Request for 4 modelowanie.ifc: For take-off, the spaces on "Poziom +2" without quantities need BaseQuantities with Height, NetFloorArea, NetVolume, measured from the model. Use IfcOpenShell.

First a look at what the model holds.

```python
import ifcopenshell
import ifcopenshell.util.element
import ifcopenshell.util.unit

model = ifcopenshell.open("4 modelowanie.ifc")
print(model.schema)
for unit_type in ("LENGTHUNIT", "AREAUNIT", "VOLUMEUNIT"):
    print(unit_type, ifcopenshell.util.unit.calculate_unit_scale(model, unit_type))
storey = next(s for s in model.by_type("IfcBuildingStorey") if s.Name == "Poziom +2")
spaces = [e for e in ifcopenshell.util.element.get_decomposition(storey) if e.is_a("IfcSpace")]
for e in sorted(spaces, key=lambda e: e.id()):
    print(e.id(), e.is_a(), e.Name, list(ifcopenshell.util.element.get_psets(e, qtos_only=True)), sep=" | ")
```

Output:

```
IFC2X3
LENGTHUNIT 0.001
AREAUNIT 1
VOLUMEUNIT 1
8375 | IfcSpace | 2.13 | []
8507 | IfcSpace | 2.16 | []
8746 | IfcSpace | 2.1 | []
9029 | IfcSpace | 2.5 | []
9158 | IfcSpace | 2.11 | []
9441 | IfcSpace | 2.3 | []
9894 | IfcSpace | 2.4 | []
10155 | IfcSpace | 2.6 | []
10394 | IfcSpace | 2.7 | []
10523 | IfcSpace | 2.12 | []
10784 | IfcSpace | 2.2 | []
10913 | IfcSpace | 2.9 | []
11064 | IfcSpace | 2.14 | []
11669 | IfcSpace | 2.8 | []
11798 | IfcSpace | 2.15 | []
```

```python
import ifcopenshell
import ifcopenshell.api.pset
import ifcopenshell.geom
import ifcopenshell.util.element
import ifcopenshell.util.shape
import ifcopenshell.util.unit

model = ifcopenshell.open("4 modelowanie.ifc")
unit_scale = ifcopenshell.util.unit.calculate_unit_scale(model)
area_scale = ifcopenshell.util.unit.calculate_unit_scale(model, "AREAUNIT")
volume_scale = ifcopenshell.util.unit.calculate_unit_scale(model, "VOLUMEUNIT")
settings = ifcopenshell.geom.settings()

storey = next(s for s in model.by_type("IfcBuildingStorey") if s.Name == "Poziom +2")
spaces = [e for e in ifcopenshell.util.element.get_decomposition(storey) if e.is_a("IfcSpace")]

for e in sorted(spaces, key=lambda e: e.id()):
    if ifcopenshell.util.element.get_psets(e, qtos_only=True, should_inherit=False):
        continue
    # Geometry comes back in metres, in the element's own axes.
    shape = ifcopenshell.geom.create_shape(settings, e)
    values = {
        "Height": ifcopenshell.util.shape.get_z(shape.geometry) / unit_scale,
        "NetFloorArea": ifcopenshell.util.shape.get_footprint_area(shape.geometry) / area_scale,
        "NetVolume": ifcopenshell.util.shape.get_volume(shape.geometry) / volume_scale,
    }
    qto = ifcopenshell.api.pset.add_qto(model, product=e, name="BaseQuantities")
    ifcopenshell.api.pset.edit_qto(model, qto=qto, properties=values)
    print(e.id(), {k: round(v, 3) for k, v in values.items()})

model.write("4 modelowanie-out.ifc")
```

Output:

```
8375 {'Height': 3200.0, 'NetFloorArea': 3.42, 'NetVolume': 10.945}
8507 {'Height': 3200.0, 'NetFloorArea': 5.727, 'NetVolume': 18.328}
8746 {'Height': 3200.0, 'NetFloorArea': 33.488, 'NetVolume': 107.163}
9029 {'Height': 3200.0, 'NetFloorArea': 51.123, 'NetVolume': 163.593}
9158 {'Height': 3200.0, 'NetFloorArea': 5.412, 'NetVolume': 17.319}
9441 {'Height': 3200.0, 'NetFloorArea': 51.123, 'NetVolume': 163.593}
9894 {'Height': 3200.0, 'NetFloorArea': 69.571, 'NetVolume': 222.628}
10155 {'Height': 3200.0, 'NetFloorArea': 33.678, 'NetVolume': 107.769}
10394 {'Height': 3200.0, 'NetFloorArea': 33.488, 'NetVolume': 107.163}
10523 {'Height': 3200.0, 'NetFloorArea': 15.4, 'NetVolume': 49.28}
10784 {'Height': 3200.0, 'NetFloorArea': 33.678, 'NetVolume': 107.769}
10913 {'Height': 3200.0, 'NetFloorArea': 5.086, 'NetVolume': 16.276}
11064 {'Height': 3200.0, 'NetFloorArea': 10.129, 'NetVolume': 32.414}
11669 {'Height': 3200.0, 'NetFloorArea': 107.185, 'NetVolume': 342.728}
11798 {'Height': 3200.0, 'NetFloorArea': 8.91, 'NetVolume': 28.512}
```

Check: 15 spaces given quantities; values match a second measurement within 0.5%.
